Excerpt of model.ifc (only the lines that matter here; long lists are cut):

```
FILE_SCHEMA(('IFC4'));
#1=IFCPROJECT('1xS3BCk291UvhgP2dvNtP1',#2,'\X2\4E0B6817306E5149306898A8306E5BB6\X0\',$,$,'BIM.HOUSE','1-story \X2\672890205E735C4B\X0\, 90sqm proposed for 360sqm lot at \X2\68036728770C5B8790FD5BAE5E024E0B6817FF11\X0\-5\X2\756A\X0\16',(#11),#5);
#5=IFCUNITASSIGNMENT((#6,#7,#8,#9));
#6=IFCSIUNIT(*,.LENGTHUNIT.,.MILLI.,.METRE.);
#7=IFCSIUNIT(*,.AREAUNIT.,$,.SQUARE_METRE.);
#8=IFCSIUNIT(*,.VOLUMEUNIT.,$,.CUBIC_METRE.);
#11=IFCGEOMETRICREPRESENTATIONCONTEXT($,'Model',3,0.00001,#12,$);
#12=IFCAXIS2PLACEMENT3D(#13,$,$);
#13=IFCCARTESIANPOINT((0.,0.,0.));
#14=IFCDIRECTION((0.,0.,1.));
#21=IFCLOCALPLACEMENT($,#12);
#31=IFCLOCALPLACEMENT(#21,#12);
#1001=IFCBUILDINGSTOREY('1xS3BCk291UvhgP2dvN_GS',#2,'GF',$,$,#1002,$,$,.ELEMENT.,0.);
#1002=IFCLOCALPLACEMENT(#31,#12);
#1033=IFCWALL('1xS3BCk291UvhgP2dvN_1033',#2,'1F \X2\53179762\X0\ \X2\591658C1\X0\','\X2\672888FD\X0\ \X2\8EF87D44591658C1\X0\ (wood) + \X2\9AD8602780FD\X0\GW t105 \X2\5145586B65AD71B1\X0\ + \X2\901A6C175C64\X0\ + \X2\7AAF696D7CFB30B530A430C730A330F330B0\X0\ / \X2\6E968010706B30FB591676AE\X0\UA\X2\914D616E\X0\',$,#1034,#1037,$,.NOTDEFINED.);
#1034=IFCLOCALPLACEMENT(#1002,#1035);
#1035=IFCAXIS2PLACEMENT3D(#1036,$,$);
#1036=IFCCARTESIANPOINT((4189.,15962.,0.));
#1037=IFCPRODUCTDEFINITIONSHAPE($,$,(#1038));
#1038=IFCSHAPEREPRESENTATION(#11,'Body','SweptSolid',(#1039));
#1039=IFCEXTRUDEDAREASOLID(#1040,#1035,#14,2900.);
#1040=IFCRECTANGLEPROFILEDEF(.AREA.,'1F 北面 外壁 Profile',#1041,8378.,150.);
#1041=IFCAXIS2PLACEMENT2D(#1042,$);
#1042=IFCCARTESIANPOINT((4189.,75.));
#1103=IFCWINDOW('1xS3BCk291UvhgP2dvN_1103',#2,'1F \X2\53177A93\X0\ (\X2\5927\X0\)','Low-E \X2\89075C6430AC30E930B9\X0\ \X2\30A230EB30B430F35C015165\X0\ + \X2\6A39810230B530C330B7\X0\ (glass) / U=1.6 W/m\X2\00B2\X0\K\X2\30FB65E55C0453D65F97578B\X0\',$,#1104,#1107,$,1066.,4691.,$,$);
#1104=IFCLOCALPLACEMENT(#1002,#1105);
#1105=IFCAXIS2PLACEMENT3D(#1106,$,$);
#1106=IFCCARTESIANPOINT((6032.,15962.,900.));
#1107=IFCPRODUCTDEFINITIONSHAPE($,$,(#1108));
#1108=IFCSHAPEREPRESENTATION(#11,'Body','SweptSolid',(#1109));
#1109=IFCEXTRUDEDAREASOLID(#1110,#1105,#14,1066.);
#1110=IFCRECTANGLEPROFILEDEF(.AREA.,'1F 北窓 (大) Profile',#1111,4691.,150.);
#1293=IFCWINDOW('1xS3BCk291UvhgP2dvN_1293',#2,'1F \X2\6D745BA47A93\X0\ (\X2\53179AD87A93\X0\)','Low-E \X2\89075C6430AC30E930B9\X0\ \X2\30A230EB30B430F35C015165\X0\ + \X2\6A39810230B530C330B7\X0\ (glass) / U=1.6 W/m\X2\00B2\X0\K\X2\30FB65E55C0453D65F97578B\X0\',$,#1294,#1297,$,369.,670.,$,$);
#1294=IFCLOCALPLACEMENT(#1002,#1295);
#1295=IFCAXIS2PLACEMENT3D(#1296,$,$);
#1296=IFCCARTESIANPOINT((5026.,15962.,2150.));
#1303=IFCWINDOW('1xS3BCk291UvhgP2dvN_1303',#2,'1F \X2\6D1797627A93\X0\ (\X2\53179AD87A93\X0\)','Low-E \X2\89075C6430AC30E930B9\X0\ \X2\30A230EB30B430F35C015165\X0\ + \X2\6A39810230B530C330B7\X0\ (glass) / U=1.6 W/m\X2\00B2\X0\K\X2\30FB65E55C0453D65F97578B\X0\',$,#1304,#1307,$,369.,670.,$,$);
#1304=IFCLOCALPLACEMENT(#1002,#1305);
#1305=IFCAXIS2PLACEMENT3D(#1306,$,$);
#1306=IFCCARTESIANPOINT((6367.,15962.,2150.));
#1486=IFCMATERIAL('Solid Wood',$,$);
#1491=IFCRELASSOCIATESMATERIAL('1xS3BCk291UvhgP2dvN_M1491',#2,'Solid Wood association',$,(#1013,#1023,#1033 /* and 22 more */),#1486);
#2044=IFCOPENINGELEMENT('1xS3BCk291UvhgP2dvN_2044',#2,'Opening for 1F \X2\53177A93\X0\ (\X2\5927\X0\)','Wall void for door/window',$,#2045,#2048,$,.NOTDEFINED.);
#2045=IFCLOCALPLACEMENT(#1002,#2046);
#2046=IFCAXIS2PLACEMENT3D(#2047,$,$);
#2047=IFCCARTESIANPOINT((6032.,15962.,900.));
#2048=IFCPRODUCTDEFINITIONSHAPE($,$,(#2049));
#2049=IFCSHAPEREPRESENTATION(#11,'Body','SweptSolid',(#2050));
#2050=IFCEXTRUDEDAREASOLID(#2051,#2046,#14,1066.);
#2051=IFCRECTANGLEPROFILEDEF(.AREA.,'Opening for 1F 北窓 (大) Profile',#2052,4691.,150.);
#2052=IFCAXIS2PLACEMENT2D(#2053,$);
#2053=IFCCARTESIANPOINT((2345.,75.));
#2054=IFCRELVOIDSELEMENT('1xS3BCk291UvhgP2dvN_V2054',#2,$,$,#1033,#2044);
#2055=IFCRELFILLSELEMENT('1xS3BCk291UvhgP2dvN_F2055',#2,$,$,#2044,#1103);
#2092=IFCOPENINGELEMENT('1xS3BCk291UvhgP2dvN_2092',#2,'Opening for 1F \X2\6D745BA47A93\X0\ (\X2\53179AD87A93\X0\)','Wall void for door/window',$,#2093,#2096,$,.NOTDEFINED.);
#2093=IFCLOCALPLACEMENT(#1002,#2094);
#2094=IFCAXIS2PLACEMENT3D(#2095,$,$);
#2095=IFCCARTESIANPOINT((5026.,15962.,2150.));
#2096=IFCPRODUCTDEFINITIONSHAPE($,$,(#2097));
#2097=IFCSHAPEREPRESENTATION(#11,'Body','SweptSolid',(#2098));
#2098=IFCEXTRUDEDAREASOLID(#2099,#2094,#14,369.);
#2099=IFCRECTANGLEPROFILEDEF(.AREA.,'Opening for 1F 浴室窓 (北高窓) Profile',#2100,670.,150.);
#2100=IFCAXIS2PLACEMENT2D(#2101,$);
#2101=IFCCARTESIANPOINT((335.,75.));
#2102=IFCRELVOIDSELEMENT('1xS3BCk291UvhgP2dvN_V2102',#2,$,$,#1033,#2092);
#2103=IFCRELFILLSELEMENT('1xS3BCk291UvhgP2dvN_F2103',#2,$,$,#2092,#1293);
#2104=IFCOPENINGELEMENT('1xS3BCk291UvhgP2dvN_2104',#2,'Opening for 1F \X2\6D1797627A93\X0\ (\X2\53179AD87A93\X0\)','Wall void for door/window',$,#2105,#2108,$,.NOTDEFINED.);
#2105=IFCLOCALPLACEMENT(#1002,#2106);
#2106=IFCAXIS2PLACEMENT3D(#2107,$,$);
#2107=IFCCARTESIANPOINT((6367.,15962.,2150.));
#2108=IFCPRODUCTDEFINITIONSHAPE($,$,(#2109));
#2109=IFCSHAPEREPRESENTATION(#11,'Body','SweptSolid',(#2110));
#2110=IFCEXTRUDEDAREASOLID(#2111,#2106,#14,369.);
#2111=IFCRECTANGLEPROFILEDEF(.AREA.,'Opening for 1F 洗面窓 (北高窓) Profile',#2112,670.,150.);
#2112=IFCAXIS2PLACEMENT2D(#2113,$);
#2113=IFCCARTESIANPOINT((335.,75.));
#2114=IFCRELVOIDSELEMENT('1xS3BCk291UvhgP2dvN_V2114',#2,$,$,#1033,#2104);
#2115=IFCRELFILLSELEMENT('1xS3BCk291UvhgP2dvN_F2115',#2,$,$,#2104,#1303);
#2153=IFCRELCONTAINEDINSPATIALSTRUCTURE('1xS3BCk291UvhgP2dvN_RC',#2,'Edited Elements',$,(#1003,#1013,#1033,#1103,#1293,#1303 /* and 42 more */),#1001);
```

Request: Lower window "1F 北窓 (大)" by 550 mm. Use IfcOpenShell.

```python
import numpy as np
import ifcopenshell
import ifcopenshell.api.geometry
import ifcopenshell.util.placement
import ifcopenshell.util.unit

model = ifcopenshell.open("model.ifc")
unit_scale = ifcopenshell.util.unit.calculate_unit_scale(model)

window = model.by_guid("1xS3BCk291UvhgP2dvN_1103")
opening = window.FillsVoids[0].RelatingOpeningElement
dz = -0.55 / unit_scale

shift = np.array([0.0, 0.0, dz])
# The window is not placed relative to its opening, so move both.
for product in (opening, window):
    matrix = ifcopenshell.util.placement.get_local_placement(product.ObjectPlacement)
    matrix[:3, 3] += shift
    ifcopenshell.api.geometry.edit_object_placement(model, product=product, matrix=matrix, is_si=False)

print(f"moved by {dz * unit_scale:+.3f} m")

model.write("model_updated.ifc")
```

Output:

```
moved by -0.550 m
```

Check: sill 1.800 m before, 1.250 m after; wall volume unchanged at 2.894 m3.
